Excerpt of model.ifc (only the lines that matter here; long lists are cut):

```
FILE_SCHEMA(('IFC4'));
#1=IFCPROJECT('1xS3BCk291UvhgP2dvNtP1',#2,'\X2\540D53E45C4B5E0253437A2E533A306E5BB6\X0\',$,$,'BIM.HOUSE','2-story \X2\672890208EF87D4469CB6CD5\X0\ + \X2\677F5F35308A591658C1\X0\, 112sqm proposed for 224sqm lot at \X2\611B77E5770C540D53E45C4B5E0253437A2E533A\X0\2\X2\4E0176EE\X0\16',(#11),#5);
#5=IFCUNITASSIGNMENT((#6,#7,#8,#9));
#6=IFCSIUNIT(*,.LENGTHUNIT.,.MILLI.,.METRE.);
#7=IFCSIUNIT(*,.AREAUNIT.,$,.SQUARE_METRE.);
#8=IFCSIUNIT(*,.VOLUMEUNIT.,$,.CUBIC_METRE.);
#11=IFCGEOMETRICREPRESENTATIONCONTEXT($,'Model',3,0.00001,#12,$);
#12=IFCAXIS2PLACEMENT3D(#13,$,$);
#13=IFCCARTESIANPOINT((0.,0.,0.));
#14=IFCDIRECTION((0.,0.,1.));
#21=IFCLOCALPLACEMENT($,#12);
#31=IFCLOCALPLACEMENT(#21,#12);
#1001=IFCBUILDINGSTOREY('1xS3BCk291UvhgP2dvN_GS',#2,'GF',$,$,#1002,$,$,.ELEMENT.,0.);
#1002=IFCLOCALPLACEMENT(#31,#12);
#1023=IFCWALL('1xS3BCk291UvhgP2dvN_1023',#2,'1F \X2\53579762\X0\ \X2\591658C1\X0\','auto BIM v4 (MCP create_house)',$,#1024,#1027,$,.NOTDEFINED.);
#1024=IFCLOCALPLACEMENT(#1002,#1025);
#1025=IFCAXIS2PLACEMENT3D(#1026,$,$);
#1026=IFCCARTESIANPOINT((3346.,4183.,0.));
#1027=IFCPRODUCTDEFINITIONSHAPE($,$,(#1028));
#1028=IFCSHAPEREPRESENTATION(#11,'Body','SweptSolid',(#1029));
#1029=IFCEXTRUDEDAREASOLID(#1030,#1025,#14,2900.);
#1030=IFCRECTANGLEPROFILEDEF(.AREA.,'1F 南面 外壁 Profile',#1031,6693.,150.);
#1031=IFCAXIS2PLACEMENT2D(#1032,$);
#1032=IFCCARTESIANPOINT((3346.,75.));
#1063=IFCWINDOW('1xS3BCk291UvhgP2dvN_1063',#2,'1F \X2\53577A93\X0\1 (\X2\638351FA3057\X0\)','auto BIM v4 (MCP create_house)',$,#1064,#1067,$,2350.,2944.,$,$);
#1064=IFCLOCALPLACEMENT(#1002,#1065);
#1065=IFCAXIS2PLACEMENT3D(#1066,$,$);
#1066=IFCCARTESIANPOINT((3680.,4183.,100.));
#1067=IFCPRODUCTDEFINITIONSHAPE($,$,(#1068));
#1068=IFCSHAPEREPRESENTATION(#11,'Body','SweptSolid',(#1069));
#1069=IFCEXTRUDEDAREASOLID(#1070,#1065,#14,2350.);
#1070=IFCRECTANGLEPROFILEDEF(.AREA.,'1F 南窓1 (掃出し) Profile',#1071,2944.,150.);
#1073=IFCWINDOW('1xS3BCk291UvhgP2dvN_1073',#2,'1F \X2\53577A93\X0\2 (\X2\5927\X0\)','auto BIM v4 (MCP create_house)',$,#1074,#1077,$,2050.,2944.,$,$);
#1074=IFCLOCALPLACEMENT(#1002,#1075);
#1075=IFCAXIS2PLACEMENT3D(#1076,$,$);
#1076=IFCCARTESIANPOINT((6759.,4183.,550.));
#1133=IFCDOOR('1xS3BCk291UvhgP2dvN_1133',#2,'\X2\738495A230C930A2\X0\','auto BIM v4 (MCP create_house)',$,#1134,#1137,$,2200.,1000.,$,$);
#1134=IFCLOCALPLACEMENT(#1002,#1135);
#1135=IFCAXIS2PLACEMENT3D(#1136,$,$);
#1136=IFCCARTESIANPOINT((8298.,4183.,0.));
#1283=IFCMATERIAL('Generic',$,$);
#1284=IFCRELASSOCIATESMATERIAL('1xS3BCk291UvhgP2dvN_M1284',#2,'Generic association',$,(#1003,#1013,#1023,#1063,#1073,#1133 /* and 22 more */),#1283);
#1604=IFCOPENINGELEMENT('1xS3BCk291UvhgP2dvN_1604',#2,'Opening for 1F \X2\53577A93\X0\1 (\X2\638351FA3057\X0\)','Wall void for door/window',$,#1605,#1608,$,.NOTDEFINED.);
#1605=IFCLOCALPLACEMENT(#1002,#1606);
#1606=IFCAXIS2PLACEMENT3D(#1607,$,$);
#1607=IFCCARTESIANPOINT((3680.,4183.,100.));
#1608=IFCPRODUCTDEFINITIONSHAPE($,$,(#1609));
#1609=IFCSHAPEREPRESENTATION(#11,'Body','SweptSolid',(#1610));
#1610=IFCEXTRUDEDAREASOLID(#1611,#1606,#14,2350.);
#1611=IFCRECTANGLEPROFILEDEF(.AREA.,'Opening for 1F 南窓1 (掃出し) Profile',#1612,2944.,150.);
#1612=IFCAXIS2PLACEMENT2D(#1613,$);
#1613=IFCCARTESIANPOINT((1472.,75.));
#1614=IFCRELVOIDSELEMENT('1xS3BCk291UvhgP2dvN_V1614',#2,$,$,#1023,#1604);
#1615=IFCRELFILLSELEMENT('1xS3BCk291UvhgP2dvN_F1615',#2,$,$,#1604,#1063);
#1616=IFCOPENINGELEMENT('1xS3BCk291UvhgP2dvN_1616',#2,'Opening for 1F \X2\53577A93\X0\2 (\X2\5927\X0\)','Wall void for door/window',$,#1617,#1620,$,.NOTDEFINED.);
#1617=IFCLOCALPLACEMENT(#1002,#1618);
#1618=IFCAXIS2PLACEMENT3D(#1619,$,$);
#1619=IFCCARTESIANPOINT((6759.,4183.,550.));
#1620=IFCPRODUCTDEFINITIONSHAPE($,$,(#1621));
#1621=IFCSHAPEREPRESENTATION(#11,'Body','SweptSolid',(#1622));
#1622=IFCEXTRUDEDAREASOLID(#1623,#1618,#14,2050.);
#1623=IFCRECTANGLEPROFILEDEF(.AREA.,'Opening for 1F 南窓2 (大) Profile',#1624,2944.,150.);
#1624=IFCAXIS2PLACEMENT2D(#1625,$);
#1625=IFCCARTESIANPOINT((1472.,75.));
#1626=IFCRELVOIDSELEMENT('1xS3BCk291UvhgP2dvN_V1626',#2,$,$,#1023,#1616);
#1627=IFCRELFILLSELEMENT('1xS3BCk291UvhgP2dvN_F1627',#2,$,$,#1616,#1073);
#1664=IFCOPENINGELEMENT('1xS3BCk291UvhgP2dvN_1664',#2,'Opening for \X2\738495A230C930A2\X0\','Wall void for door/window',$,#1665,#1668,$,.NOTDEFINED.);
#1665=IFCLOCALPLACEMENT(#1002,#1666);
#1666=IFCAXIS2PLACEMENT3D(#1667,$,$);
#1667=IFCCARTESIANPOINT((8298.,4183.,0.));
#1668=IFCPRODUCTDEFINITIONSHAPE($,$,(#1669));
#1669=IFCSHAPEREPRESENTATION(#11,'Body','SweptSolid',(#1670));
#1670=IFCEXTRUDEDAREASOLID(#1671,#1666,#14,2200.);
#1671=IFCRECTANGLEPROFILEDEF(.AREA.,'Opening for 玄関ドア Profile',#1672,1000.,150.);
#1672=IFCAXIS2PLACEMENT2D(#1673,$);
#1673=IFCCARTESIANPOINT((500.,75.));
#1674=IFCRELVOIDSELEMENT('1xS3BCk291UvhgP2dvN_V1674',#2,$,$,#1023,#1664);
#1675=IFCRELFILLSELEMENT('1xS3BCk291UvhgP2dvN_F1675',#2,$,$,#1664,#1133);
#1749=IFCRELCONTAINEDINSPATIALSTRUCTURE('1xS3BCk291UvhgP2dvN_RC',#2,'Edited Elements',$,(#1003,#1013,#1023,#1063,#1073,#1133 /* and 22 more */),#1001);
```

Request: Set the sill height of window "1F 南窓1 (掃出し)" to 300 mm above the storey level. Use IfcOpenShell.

```python
import numpy as np
import ifcopenshell
import ifcopenshell.api.geometry
import ifcopenshell.geom
import ifcopenshell.util.element
import ifcopenshell.util.placement
import ifcopenshell.util.shape
import ifcopenshell.util.unit

model = ifcopenshell.open("model.ifc")
unit_scale = ifcopenshell.util.unit.calculate_unit_scale(model)

window = model.by_guid("1xS3BCk291UvhgP2dvN_1063")
opening = window.FillsVoids[0].RelatingOpeningElement
storey = ifcopenshell.util.element.get_container(window, ifc_class="IfcBuildingStorey")
level = ifcopenshell.util.placement.get_local_placement(storey.ObjectPlacement)[2, 3]

# The opening's origin need not be at the sill, so measure its lowest point.
shape = ifcopenshell.geom.create_shape(ifcopenshell.geom.settings(), opening)
bottom = ifcopenshell.util.shape.get_shape_bottom_elevation(shape, shape.geometry) / unit_scale
dz = level + 0.3 / unit_scale - bottom

shift = np.array([0.0, 0.0, dz])
# The window is not placed relative to its opening, so move both.
for product in (opening, window):
    matrix = ifcopenshell.util.placement.get_local_placement(product.ObjectPlacement)
    matrix[:3, 3] += shift
    ifcopenshell.api.geometry.edit_object_placement(model, product=product, matrix=matrix, is_si=False)

print(f"moved by {dz * unit_scale:+.3f} m")

model.write("model_edited.ifc")
```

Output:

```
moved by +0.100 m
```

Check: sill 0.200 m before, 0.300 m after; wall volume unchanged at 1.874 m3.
